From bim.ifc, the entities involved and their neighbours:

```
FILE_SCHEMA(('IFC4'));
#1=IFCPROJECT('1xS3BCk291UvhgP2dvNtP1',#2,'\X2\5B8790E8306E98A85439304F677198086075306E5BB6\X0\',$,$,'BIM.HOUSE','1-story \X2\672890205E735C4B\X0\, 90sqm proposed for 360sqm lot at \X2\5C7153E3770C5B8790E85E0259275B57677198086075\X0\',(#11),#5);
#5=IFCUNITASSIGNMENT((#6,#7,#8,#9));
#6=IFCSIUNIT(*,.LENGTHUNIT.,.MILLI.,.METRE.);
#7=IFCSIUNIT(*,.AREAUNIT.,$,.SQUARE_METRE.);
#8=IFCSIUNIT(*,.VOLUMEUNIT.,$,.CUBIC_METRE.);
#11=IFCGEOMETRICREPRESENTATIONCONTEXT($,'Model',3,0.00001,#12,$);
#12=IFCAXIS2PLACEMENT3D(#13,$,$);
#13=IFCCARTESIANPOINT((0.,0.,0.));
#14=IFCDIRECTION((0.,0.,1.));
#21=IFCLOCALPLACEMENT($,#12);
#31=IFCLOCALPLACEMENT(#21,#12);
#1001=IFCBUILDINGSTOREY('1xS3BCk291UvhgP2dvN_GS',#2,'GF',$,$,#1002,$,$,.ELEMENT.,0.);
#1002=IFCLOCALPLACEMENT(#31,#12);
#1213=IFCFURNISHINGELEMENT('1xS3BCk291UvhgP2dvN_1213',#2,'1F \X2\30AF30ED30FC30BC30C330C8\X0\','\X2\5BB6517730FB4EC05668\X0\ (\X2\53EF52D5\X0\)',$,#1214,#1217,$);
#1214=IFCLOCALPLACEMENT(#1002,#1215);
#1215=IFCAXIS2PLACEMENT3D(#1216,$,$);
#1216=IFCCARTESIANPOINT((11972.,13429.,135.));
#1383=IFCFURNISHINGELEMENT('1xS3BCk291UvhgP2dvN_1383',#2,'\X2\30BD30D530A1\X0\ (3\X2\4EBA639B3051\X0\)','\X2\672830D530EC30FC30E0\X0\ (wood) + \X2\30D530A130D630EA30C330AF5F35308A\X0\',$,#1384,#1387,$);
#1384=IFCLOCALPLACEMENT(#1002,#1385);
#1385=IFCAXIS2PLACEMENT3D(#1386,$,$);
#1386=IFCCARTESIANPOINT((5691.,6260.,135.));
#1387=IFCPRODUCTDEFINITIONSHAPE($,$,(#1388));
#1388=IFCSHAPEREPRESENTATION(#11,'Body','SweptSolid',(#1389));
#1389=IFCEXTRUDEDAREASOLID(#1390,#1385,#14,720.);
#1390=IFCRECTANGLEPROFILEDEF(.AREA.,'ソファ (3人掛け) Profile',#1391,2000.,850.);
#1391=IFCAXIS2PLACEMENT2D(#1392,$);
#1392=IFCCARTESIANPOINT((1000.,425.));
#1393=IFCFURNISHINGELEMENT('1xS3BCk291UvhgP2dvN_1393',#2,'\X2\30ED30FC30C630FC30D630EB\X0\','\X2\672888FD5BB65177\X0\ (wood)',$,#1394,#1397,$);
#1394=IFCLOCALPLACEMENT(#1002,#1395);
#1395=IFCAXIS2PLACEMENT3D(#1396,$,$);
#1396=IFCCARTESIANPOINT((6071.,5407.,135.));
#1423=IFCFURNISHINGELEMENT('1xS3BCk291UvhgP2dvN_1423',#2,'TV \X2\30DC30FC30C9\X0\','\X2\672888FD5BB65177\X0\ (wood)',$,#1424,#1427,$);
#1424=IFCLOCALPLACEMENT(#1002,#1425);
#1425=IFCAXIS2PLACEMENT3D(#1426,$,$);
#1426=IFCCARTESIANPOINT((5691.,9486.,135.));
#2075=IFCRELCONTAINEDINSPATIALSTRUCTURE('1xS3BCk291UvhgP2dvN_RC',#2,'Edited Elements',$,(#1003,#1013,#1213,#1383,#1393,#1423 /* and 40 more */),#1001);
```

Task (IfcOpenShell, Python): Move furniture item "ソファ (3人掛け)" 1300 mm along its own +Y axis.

```python
import ifcopenshell
import ifcopenshell.api.geometry
import ifcopenshell.util.placement
import ifcopenshell.util.unit

model = ifcopenshell.open("bim.ifc")
unit_scale = ifcopenshell.util.unit.calculate_unit_scale(model)

item = model.by_guid("1xS3BCk291UvhgP2dvN_1383")
matrix = ifcopenshell.util.placement.get_local_placement(item.ObjectPlacement)
matrix[:3, 3] += matrix[:3, 1] * 1.3 / unit_scale
ifcopenshell.api.geometry.edit_object_placement(model, product=item, matrix=matrix, is_si=False)

print(ifcopenshell.util.placement.get_local_placement(item.ObjectPlacement).round(3) + 0.0)

model.write("bim_updated.ifc")
```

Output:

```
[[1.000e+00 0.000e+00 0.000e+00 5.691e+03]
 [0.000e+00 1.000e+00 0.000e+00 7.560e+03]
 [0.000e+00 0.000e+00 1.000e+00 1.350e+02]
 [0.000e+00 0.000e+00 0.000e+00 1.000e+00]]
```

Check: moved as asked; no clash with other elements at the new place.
